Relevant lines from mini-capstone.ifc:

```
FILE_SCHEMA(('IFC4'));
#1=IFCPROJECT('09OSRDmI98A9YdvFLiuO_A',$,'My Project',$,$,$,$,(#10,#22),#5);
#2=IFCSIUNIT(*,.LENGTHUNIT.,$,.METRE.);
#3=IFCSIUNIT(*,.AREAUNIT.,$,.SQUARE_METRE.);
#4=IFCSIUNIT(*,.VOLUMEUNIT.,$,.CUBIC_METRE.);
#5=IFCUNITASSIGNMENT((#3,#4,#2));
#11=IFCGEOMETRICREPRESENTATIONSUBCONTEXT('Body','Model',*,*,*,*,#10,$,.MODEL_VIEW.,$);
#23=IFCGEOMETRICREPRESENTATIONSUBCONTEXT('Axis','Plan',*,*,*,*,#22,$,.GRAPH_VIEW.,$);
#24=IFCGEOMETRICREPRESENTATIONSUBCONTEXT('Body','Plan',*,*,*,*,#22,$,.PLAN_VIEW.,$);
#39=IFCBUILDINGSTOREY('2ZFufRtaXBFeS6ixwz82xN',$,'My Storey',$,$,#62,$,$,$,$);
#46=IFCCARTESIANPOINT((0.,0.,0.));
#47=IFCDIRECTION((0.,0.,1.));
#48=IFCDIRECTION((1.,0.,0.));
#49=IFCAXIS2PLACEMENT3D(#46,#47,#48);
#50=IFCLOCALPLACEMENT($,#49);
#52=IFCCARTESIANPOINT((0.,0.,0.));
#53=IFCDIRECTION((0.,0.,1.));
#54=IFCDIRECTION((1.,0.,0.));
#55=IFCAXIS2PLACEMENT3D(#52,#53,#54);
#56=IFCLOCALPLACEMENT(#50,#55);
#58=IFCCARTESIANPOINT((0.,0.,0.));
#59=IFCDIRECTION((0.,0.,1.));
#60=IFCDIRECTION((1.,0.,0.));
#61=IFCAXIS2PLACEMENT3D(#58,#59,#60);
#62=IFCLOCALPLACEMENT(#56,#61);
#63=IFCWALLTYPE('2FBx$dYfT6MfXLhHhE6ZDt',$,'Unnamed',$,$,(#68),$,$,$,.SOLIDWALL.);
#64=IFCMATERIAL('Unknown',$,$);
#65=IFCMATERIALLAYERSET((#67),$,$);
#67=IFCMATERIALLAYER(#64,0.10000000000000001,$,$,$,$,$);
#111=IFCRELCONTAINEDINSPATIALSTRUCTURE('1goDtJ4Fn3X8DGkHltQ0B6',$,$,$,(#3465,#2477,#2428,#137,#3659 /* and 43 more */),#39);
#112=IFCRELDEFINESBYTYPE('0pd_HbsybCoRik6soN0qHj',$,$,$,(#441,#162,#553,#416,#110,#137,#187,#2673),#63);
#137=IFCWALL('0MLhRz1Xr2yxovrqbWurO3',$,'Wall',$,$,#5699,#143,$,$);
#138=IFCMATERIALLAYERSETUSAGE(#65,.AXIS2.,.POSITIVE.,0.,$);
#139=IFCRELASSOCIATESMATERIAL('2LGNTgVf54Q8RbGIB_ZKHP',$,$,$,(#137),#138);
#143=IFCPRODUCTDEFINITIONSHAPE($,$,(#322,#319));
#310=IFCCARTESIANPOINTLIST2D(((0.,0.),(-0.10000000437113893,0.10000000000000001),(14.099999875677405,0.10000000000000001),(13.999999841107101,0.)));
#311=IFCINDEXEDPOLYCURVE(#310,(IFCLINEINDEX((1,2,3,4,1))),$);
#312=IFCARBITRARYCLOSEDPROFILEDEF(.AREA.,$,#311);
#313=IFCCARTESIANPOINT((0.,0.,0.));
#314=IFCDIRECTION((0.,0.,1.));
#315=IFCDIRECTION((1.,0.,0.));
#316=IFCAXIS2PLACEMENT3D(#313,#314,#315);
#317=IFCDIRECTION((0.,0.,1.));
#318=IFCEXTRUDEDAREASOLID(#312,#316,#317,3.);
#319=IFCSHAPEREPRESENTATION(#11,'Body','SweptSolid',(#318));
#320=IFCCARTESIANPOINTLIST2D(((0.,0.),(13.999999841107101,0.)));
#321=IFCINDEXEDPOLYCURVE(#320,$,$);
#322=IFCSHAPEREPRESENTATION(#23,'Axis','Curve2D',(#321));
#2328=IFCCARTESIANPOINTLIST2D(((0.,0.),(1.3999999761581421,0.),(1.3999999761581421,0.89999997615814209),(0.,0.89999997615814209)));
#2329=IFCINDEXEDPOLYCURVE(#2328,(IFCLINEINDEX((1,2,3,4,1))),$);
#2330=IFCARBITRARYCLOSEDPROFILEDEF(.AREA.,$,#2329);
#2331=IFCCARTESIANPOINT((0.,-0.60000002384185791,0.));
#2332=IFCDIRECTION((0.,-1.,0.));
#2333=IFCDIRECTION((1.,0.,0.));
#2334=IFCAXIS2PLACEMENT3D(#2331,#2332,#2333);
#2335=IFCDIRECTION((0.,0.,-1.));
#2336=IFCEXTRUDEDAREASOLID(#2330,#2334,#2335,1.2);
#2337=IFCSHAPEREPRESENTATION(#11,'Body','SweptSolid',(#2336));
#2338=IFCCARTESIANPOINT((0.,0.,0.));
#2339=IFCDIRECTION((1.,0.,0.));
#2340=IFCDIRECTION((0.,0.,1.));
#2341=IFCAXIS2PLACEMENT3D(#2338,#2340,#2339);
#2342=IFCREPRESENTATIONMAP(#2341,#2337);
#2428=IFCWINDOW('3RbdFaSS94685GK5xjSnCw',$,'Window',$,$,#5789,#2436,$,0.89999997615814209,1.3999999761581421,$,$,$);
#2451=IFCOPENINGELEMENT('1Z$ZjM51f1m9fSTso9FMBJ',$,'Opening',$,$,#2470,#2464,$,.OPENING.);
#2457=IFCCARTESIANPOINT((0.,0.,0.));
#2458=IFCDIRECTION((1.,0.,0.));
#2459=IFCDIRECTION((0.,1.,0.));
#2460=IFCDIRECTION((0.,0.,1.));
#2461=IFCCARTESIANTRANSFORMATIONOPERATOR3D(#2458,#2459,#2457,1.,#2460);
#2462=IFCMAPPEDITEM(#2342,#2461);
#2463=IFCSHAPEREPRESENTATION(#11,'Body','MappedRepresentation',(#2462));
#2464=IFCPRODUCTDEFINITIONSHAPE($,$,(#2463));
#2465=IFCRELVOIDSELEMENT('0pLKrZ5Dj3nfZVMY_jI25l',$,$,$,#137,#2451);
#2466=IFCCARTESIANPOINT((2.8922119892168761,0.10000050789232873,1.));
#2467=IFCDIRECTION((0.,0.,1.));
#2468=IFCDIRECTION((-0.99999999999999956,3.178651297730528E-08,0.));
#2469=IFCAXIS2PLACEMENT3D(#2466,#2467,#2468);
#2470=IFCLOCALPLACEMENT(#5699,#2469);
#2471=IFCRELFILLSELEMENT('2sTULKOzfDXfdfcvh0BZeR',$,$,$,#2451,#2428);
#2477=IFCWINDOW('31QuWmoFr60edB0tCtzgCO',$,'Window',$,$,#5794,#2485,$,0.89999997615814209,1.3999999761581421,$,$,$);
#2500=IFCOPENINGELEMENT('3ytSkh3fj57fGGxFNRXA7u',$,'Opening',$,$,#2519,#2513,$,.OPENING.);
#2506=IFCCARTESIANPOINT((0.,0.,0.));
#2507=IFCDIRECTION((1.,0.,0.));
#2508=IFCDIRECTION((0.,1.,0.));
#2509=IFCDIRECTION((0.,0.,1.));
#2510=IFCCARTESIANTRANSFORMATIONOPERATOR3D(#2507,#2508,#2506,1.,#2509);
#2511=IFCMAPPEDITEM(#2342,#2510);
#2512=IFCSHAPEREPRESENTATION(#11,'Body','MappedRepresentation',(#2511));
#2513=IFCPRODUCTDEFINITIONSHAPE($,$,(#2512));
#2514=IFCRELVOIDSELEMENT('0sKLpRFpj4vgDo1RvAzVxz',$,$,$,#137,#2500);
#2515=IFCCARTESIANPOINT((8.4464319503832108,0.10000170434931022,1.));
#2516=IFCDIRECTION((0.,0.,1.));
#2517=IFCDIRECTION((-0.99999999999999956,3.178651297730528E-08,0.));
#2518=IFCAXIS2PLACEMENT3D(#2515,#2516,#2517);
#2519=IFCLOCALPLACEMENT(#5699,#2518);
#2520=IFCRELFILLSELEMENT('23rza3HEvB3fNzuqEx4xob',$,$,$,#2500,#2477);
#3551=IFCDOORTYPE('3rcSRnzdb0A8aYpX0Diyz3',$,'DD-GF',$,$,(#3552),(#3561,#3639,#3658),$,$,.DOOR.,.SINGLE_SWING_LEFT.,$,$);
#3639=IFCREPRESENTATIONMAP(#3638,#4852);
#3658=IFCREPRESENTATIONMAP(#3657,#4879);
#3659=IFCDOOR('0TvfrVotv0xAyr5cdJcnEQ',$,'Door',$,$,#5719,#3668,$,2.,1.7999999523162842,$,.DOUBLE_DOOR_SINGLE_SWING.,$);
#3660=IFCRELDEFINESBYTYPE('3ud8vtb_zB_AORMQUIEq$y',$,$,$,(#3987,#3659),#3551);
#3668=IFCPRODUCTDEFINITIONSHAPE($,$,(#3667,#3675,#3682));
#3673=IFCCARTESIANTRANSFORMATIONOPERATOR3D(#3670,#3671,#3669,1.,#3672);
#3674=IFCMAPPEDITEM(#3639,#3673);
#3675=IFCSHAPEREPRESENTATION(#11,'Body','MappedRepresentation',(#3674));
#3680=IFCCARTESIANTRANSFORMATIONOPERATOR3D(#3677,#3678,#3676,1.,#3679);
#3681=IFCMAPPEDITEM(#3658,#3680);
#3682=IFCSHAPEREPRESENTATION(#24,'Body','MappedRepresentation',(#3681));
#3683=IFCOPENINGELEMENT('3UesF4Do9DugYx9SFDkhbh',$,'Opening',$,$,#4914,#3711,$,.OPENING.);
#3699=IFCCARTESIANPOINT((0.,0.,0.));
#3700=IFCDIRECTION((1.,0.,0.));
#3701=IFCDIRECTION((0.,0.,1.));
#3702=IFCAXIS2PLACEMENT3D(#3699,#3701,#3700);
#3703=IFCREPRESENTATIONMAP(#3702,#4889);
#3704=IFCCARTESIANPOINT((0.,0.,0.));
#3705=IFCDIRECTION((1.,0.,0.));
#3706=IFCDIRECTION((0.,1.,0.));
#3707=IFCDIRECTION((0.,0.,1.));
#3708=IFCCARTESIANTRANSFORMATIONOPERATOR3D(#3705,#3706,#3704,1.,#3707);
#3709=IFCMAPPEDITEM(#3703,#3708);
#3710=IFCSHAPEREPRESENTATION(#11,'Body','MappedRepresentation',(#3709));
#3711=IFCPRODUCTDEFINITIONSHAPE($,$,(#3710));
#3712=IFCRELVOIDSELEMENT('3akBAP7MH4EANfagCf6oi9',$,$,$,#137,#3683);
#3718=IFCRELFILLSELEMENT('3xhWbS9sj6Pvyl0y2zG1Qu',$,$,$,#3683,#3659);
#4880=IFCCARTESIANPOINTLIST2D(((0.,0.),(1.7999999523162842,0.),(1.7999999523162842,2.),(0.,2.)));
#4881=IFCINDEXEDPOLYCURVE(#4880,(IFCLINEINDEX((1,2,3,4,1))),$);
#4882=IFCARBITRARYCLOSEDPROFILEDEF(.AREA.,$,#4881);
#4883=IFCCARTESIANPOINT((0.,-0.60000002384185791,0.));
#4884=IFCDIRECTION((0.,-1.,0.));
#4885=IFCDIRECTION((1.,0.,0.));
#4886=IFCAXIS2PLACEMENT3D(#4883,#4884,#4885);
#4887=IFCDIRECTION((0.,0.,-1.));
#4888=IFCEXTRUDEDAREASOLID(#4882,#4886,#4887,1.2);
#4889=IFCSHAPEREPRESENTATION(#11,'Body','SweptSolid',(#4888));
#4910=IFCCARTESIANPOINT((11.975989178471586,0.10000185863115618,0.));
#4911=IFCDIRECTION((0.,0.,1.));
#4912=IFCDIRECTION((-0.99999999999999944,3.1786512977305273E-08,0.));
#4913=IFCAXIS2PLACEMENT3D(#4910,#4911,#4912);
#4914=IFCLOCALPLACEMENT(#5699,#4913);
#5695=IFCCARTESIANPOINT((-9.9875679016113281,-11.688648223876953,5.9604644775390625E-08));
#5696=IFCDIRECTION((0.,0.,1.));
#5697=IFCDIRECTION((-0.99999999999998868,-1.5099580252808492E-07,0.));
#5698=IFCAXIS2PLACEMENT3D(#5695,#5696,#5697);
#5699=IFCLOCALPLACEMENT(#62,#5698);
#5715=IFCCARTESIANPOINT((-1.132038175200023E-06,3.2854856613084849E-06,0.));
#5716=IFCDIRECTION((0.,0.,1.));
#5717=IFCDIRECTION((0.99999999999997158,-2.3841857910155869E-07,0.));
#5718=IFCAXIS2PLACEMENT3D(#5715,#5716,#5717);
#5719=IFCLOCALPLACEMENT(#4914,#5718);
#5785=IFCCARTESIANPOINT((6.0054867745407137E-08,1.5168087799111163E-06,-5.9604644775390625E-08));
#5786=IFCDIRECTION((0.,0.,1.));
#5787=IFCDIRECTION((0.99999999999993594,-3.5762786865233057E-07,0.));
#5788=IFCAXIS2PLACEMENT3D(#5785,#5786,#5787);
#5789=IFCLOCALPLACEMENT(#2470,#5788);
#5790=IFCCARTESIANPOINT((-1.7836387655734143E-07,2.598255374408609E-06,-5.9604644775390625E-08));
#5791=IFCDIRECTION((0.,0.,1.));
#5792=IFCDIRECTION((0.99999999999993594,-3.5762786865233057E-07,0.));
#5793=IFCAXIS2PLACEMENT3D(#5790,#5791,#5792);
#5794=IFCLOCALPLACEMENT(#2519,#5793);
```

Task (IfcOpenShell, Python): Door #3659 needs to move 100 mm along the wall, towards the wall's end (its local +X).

```python
import ifcopenshell
import ifcopenshell.api.geometry
import ifcopenshell.util.placement

model = ifcopenshell.open("mini-capstone.ifc")

door = model.by_id(3659)
opening = door.FillsVoids[0].RelatingOpeningElement
wall = opening.VoidsElements[0].RelatingBuildingElement

wall_matrix = ifcopenshell.util.placement.get_local_placement(wall.ObjectPlacement)
shift = wall_matrix[:3, 0] * 0.1
before = ifcopenshell.util.placement.get_local_placement(door.ObjectPlacement)[:3, 3].copy()

# The door is placed relative to its opening, so it follows when the opening moves.
matrix = ifcopenshell.util.placement.get_local_placement(opening.ObjectPlacement)
matrix[:3, 3] += shift
ifcopenshell.api.geometry.edit_object_placement(
    model, product=opening, matrix=matrix, is_si=False, should_transform_children=True
)

after = ifcopenshell.util.placement.get_local_placement(door.ObjectPlacement)[:3, 3]
print("door moved by", (after - before).round(3) + 0.0)

model.write("mini-capstone-out.ifc")
```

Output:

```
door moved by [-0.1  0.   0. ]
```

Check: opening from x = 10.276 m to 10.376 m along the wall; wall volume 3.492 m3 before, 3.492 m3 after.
